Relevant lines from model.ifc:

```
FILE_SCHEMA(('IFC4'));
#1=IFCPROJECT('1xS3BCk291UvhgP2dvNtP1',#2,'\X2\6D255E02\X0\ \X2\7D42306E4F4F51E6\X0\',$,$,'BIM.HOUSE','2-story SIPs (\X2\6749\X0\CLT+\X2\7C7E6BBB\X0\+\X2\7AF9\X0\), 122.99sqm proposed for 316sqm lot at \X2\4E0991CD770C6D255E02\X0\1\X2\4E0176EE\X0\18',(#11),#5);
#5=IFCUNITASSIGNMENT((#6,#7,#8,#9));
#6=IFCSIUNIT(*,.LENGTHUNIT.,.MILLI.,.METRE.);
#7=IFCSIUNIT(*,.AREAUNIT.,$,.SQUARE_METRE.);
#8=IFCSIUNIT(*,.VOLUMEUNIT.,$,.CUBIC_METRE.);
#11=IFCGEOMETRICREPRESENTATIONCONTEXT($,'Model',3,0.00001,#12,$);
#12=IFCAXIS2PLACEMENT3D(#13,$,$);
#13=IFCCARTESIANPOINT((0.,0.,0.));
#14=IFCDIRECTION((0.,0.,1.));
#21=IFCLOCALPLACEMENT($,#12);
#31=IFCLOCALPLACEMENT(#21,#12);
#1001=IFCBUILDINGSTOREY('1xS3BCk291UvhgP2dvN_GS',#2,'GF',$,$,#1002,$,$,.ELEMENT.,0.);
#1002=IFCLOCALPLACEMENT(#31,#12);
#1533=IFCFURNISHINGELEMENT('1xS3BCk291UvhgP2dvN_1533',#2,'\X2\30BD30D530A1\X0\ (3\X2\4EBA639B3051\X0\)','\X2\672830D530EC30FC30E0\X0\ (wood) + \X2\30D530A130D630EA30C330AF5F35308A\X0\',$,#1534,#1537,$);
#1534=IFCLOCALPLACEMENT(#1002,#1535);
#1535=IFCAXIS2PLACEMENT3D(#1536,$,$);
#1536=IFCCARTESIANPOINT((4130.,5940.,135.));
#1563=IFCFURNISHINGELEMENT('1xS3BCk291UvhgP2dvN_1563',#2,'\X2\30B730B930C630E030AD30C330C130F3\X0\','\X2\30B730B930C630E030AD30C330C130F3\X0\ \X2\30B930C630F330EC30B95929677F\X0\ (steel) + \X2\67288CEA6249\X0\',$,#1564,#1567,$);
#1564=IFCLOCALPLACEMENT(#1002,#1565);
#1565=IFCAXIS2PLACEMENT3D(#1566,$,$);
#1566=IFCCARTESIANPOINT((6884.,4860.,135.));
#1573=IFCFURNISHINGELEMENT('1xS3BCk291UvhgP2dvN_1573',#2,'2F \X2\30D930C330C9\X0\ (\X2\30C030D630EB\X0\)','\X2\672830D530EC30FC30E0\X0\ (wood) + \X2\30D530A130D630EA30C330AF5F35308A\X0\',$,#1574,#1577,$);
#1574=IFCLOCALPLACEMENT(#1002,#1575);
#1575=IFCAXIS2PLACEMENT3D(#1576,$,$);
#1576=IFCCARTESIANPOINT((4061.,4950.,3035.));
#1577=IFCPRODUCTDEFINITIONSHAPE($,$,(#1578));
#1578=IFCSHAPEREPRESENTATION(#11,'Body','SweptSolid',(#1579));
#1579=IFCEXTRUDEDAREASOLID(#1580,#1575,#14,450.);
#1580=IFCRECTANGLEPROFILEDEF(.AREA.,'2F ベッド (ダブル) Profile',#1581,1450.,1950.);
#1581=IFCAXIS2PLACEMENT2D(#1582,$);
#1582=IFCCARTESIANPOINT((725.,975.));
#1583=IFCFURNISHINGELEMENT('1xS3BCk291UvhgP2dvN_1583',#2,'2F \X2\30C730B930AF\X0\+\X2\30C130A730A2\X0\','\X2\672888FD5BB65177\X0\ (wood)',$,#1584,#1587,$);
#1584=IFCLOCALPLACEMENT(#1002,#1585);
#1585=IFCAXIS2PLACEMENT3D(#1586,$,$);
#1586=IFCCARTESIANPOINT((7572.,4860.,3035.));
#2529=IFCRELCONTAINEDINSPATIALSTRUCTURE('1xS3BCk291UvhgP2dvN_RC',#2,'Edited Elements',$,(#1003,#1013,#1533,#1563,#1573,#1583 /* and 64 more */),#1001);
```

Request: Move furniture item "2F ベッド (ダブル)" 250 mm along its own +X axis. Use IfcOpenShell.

```python
import ifcopenshell
import ifcopenshell.api.geometry
import ifcopenshell.util.placement
import ifcopenshell.util.unit

model = ifcopenshell.open("model.ifc")
unit_scale = ifcopenshell.util.unit.calculate_unit_scale(model)

item = model.by_guid("1xS3BCk291UvhgP2dvN_1573")
matrix = ifcopenshell.util.placement.get_local_placement(item.ObjectPlacement)
matrix[:3, 3] += matrix[:3, 0] * 0.25 / unit_scale
ifcopenshell.api.geometry.edit_object_placement(model, product=item, matrix=matrix, is_si=False)

print(ifcopenshell.util.placement.get_local_placement(item.ObjectPlacement).round(3) + 0.0)

model.write("model_v2.ifc")
```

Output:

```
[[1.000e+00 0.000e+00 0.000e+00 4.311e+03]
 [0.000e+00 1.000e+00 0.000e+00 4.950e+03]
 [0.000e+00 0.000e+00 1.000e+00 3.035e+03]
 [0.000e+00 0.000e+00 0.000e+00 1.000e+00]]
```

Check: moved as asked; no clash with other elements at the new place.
